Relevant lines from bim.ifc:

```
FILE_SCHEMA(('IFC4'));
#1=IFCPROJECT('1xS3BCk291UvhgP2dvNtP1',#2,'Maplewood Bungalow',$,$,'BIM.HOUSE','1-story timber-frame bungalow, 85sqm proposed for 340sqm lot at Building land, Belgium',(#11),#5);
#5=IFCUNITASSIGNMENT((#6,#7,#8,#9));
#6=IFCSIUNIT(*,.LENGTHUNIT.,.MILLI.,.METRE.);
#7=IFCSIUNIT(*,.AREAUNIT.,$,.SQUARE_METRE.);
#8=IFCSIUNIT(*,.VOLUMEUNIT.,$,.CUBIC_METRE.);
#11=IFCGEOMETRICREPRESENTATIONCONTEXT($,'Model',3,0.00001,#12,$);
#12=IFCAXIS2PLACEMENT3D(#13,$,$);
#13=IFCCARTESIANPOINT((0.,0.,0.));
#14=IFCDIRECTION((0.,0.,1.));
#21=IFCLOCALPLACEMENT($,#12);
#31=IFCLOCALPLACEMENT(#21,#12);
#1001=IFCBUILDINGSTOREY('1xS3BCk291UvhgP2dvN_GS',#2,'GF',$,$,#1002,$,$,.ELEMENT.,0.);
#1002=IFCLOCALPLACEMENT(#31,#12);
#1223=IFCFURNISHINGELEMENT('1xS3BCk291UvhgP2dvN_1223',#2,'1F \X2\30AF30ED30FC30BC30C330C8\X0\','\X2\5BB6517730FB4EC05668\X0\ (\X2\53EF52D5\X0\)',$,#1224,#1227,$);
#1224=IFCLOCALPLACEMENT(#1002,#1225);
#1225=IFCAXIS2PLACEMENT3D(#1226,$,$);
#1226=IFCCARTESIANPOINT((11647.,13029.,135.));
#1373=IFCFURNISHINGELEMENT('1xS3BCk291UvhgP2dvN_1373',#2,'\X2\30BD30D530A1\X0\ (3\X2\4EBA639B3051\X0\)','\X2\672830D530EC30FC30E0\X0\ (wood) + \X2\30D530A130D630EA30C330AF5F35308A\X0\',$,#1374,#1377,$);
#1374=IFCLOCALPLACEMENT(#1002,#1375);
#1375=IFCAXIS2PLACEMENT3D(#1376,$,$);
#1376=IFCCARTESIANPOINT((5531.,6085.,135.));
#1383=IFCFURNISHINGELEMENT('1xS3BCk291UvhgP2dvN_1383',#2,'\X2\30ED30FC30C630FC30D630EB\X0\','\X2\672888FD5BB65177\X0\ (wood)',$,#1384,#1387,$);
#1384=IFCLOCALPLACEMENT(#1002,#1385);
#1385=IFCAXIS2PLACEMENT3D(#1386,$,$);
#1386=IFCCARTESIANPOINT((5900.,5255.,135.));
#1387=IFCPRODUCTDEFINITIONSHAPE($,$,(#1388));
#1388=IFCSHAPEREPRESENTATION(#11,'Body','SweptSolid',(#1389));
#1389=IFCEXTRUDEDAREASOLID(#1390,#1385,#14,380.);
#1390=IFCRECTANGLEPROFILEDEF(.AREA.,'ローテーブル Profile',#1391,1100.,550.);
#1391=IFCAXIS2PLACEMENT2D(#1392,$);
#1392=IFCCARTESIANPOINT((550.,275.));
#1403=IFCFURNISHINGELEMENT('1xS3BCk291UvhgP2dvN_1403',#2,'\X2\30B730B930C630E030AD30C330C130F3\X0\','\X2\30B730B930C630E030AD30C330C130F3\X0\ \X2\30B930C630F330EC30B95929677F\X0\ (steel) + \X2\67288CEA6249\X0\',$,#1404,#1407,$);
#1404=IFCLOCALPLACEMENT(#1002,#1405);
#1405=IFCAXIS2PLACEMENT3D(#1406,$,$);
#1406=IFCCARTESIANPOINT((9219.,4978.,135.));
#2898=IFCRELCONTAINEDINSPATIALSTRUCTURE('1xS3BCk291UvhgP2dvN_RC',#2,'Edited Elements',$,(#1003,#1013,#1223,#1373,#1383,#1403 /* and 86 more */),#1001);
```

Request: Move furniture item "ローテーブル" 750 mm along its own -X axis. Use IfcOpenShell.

```python
import ifcopenshell
import ifcopenshell.api.geometry
import ifcopenshell.util.placement
import ifcopenshell.util.unit

model = ifcopenshell.open("bim.ifc")
unit_scale = ifcopenshell.util.unit.calculate_unit_scale(model)

item = model.by_id(1383)
matrix = ifcopenshell.util.placement.get_local_placement(item.ObjectPlacement)
matrix[:3, 3] -= matrix[:3, 0] * 0.75 / unit_scale
ifcopenshell.api.geometry.edit_object_placement(model, product=item, matrix=matrix, is_si=False)

print(ifcopenshell.util.placement.get_local_placement(item.ObjectPlacement).round(3) + 0.0)

model.write("bim_updated.ifc")
```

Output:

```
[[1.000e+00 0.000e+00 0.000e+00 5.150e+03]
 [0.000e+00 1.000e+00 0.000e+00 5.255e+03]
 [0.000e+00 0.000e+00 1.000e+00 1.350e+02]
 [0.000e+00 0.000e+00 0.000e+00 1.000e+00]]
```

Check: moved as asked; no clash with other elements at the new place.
